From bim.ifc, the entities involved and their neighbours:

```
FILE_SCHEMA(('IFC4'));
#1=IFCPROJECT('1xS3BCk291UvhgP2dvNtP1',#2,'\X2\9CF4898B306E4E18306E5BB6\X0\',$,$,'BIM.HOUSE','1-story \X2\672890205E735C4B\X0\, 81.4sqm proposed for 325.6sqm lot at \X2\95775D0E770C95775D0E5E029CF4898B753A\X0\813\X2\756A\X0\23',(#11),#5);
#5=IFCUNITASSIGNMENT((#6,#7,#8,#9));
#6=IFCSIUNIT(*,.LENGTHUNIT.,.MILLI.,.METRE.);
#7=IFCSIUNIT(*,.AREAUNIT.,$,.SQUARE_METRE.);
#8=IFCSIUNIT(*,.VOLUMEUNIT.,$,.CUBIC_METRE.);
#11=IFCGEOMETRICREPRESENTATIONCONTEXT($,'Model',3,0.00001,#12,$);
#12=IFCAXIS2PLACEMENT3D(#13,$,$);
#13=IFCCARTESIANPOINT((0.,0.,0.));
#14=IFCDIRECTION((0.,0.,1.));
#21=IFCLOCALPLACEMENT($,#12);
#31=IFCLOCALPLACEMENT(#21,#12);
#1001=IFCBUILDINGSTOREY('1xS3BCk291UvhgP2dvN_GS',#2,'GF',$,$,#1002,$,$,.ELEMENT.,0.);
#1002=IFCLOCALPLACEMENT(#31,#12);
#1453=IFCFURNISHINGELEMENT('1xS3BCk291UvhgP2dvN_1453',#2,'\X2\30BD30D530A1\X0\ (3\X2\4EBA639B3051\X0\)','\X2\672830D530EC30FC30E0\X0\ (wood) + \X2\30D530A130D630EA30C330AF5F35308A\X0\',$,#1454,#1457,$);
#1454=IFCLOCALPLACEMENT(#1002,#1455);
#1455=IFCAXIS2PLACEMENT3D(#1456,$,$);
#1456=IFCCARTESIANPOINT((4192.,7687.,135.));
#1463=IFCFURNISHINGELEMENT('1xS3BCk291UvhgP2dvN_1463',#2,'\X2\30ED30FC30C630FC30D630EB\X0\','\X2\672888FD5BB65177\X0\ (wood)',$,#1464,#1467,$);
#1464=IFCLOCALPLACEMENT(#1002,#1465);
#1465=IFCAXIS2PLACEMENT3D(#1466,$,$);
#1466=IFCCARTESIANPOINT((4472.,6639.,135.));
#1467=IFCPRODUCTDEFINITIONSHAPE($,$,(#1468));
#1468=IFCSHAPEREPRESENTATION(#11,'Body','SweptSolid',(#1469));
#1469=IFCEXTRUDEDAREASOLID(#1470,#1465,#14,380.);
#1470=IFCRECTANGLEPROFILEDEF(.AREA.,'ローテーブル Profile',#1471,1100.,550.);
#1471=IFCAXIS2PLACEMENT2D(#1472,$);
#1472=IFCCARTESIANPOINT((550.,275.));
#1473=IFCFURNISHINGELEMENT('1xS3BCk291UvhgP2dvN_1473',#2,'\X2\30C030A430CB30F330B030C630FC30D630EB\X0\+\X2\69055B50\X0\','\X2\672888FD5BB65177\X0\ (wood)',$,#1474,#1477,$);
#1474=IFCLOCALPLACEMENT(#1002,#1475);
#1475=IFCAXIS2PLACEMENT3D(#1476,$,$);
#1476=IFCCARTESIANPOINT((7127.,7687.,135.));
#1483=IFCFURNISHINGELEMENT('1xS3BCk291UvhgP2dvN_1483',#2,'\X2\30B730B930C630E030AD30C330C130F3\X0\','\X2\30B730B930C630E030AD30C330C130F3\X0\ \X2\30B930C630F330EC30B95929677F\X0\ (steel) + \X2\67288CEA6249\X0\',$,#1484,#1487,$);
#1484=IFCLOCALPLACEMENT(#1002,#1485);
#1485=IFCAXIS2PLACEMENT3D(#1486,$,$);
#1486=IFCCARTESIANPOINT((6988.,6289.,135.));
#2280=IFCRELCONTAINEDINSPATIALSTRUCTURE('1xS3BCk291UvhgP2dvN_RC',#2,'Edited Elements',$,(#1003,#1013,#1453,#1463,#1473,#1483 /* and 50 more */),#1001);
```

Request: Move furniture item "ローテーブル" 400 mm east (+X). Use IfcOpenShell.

```python
import ifcopenshell
import ifcopenshell.api.geometry
import ifcopenshell.util.placement
import ifcopenshell.util.unit

model = ifcopenshell.open("bim.ifc")
unit_scale = ifcopenshell.util.unit.calculate_unit_scale(model)

item = model.by_guid("1xS3BCk291UvhgP2dvN_1463")
matrix = ifcopenshell.util.placement.get_local_placement(item.ObjectPlacement)
matrix[0, 3] += 0.4 / unit_scale
ifcopenshell.api.geometry.edit_object_placement(model, product=item, matrix=matrix, is_si=False)

print(ifcopenshell.util.placement.get_local_placement(item.ObjectPlacement).round(3) + 0.0)

model.write("bim-out.ifc")
```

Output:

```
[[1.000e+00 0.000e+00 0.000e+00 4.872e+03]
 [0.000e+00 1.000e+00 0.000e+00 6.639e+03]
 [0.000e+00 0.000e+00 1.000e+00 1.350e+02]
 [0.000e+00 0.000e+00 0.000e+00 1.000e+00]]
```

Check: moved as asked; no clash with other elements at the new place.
